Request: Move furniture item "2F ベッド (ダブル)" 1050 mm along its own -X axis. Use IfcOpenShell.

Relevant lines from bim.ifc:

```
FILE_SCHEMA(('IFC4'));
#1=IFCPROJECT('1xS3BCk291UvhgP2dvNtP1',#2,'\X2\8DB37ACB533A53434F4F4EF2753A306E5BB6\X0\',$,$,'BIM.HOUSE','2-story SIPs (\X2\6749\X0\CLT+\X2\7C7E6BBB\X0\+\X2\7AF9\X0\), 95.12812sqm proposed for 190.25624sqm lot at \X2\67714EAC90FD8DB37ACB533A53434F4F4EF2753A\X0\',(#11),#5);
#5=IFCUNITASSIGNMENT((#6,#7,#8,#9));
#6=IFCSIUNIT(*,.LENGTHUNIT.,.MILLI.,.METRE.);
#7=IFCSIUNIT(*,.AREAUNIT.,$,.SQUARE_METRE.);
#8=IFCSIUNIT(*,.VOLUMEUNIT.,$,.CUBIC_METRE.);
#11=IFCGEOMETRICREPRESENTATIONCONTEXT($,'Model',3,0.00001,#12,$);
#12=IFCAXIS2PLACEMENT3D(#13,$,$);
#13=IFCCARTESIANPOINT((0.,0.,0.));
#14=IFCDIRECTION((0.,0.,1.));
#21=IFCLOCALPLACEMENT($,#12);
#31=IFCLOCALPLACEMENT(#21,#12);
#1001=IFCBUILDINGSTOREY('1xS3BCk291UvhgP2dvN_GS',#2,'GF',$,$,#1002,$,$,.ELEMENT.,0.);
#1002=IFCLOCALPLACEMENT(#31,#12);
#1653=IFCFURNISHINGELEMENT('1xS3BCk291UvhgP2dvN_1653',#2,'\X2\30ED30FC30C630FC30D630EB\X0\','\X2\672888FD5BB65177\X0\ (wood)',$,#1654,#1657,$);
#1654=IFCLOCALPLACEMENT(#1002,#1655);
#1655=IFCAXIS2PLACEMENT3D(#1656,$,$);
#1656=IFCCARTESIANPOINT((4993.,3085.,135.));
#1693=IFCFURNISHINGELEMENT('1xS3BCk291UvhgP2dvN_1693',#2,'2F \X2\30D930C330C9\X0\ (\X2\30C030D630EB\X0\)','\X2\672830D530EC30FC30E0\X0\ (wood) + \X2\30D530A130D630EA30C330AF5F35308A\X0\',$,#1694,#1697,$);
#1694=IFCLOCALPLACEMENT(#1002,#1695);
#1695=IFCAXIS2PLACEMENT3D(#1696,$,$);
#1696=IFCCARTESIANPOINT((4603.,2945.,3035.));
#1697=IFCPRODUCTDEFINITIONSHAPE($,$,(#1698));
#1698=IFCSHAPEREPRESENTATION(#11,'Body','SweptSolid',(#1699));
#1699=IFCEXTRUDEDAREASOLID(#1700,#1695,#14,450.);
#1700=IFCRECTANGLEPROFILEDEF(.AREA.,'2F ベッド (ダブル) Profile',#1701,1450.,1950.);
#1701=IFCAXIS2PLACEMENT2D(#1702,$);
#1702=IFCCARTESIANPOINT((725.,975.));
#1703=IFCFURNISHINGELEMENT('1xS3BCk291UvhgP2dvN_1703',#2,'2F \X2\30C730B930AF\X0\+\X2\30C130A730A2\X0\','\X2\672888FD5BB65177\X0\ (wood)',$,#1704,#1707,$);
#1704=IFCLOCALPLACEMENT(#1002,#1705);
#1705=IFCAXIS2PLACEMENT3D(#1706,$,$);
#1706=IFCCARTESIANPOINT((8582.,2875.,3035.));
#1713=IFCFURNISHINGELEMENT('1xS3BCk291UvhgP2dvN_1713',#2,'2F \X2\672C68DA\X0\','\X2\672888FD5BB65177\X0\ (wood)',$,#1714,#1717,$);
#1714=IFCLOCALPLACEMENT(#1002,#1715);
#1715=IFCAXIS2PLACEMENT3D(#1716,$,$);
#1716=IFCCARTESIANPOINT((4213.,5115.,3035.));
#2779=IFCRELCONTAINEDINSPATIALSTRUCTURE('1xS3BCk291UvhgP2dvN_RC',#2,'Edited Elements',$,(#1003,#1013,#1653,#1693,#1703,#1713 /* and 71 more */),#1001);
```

```python
import ifcopenshell
import ifcopenshell.api.geometry
import ifcopenshell.util.placement
import ifcopenshell.util.unit

model = ifcopenshell.open("bim.ifc")
unit_scale = ifcopenshell.util.unit.calculate_unit_scale(model)

item = model.by_guid("1xS3BCk291UvhgP2dvN_1693")
matrix = ifcopenshell.util.placement.get_local_placement(item.ObjectPlacement)
matrix[:3, 3] -= matrix[:3, 0] * 1.05 / unit_scale
ifcopenshell.api.geometry.edit_object_placement(model, product=item, matrix=matrix, is_si=False)

print(ifcopenshell.util.placement.get_local_placement(item.ObjectPlacement).round(3) + 0.0)

model.write("bim_updated.ifc")
```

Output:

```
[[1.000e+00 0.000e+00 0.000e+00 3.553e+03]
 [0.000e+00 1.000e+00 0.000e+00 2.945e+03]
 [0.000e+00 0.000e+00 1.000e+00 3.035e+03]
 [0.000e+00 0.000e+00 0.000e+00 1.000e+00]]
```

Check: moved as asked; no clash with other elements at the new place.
